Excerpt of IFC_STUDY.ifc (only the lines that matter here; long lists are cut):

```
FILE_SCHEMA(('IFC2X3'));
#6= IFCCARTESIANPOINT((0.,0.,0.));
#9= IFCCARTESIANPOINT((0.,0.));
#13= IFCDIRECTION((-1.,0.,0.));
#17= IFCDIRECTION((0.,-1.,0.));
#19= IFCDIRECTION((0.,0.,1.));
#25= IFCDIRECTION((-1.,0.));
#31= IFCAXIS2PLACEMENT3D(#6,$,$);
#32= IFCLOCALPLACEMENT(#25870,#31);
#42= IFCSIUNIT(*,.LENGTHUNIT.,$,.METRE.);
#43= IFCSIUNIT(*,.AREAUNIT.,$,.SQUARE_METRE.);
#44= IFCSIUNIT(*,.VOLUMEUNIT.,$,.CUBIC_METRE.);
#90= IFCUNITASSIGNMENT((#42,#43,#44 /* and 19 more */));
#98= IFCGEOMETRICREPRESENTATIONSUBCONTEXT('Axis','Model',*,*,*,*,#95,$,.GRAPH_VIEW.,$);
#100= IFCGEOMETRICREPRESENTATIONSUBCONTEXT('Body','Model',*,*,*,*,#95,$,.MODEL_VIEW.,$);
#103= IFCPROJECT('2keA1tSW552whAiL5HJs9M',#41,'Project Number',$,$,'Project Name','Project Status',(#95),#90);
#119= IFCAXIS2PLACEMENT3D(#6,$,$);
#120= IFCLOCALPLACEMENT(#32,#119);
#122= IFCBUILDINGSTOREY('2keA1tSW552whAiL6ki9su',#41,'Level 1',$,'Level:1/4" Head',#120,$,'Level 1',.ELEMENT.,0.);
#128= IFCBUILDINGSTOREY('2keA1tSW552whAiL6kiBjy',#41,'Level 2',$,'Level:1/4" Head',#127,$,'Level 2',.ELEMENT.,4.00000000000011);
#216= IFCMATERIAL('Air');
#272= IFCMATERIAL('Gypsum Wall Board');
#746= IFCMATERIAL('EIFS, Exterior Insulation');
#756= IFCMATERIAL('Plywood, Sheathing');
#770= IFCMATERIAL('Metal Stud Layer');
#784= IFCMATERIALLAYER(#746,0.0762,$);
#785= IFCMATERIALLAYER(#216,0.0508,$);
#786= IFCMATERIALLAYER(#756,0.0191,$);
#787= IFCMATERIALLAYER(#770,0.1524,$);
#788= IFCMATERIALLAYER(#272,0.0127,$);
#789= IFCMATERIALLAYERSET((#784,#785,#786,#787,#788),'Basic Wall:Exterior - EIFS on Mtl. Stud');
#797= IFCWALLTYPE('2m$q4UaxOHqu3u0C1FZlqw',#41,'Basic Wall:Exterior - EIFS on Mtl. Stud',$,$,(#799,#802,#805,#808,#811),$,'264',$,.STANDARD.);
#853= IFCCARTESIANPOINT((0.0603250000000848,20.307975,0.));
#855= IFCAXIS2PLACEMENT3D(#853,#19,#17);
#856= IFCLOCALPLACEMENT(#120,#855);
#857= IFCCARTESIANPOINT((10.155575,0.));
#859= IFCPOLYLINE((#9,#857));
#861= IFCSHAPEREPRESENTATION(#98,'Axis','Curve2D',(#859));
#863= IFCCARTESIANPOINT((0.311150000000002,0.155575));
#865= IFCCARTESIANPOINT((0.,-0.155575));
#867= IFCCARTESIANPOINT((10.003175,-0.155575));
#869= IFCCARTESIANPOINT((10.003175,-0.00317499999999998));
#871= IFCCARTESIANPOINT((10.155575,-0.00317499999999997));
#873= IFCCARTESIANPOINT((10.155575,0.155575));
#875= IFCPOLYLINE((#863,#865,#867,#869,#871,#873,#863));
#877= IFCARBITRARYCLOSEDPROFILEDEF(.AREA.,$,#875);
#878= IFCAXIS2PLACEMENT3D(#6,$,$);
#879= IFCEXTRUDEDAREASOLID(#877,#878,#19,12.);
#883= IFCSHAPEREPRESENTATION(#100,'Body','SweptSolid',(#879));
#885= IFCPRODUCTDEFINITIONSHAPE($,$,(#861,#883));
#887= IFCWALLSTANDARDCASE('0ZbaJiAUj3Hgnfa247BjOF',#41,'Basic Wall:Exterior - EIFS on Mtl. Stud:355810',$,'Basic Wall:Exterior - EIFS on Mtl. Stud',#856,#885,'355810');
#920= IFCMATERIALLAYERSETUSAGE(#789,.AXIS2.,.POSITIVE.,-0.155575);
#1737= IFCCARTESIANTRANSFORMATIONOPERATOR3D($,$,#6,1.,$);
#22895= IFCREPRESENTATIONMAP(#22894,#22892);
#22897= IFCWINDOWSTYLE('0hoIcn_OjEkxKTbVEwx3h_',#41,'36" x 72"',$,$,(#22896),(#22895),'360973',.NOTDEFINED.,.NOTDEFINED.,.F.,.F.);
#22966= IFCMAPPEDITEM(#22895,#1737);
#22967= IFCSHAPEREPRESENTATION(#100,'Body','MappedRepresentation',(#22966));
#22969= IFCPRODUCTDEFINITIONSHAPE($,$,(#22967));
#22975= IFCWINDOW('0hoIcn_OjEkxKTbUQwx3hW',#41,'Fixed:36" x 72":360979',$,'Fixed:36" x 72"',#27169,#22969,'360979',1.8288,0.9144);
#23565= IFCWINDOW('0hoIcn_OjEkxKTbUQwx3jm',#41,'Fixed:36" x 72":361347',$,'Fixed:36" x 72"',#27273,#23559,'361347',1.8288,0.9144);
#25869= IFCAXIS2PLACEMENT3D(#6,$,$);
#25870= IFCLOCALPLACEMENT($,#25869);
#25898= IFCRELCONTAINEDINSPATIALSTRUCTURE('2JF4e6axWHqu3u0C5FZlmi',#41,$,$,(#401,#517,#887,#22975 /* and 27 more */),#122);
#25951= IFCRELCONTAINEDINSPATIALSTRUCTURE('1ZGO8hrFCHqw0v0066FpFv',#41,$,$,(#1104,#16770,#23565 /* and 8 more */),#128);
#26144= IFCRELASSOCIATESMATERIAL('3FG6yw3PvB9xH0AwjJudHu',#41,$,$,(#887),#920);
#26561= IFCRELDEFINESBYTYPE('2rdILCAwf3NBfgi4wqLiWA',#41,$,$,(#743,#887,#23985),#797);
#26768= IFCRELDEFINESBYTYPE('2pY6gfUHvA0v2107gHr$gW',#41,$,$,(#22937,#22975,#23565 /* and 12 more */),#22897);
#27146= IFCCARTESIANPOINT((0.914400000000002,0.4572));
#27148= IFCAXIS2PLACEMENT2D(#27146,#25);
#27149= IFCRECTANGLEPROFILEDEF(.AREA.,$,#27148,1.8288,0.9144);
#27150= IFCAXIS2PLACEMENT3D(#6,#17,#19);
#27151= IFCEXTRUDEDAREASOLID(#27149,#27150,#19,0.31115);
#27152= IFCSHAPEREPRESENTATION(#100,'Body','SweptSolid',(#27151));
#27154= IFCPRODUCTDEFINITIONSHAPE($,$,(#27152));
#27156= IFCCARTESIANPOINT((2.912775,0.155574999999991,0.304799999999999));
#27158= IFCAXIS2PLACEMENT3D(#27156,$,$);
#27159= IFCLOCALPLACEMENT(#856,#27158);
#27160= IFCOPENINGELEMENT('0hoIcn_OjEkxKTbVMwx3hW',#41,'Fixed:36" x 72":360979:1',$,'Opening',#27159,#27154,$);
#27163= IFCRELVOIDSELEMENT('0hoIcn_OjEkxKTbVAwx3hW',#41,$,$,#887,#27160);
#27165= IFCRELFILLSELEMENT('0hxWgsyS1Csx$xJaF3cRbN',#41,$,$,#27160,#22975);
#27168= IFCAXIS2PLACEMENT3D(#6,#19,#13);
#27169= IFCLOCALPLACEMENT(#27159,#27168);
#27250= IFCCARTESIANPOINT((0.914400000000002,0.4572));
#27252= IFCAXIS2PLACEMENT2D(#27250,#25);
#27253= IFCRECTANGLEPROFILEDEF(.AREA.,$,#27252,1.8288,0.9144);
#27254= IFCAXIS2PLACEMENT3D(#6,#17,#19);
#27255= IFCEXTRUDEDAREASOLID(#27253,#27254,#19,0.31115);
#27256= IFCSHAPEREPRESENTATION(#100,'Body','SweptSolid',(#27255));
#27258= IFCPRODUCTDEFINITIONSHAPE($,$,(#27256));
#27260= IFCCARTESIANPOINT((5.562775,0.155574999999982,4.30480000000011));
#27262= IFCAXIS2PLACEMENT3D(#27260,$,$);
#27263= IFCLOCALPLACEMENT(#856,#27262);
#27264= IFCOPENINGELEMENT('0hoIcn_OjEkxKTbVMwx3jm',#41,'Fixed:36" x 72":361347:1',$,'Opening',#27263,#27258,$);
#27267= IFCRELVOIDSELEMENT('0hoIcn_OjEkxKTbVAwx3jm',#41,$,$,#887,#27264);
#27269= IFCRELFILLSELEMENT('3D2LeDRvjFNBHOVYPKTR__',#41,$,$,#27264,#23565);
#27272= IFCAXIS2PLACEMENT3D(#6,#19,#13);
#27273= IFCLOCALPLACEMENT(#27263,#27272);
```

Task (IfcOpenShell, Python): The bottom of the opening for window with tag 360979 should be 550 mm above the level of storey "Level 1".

```python
import numpy as np
import ifcopenshell
import ifcopenshell.api.geometry
import ifcopenshell.geom
import ifcopenshell.util.element
import ifcopenshell.util.placement
import ifcopenshell.util.shape
import ifcopenshell.util.unit

model = ifcopenshell.open("IFC_STUDY.ifc")
unit_scale = ifcopenshell.util.unit.calculate_unit_scale(model)

window = model.by_guid("0hoIcn_OjEkxKTbUQwx3hW")
opening = window.FillsVoids[0].RelatingOpeningElement
storey = ifcopenshell.util.element.get_container(window, ifc_class="IfcBuildingStorey")
level = ifcopenshell.util.placement.get_local_placement(storey.ObjectPlacement)[2, 3]

# The opening's origin need not be at the sill, so measure its lowest point.
shape = ifcopenshell.geom.create_shape(ifcopenshell.geom.settings(), opening)
bottom = ifcopenshell.util.shape.get_shape_bottom_elevation(shape, shape.geometry) / unit_scale
dz = level + 0.55 - bottom

shift = np.array([0.0, 0.0, dz])
# The window is placed relative to its opening, so it follows when the opening moves.
matrix = ifcopenshell.util.placement.get_local_placement(opening.ObjectPlacement)
matrix[:3, 3] += shift
ifcopenshell.api.geometry.edit_object_placement(
    model, product=opening, matrix=matrix, is_si=False, should_transform_children=True
)

print(f"moved by {dz * unit_scale:+.3f} m")

model.write("IFC_STUDY_v2.ifc")
```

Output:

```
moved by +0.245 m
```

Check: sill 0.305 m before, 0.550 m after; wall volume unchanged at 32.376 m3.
